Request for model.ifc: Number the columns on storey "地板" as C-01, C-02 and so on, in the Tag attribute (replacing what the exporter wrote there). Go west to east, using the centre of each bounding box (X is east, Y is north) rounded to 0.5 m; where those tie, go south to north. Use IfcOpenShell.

First a look at what the model holds.

```python
import ifcopenshell
import ifcopenshell.util.element
import ifcopenshell.util.placement

model = ifcopenshell.open("model.ifc")
print(model.schema)
storey = next(s for s in model.by_type("IfcBuildingStorey") if s.Name == "地板")
columns = [e for e in ifcopenshell.util.element.get_decomposition(storey) if e.is_a("IfcColumn")]
for e in sorted(columns, key=lambda e: e.id()):
    origin = ifcopenshell.util.placement.get_local_placement(e.ObjectPlacement)[:3, 3]
    print(e.id(), e.Tag, e.Name, origin.round(2) + 0.0, sep=" | ")
```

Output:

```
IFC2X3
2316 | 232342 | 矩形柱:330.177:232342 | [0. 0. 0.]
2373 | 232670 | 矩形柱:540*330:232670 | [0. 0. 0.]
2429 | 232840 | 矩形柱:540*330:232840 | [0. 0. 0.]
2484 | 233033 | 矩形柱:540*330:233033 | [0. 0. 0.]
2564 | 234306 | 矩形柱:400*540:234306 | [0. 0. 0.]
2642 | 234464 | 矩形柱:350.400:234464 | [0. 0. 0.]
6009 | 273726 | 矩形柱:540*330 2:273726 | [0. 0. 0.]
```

```python
import ifcopenshell
import ifcopenshell.geom
import ifcopenshell.util.element
import ifcopenshell.util.shape

model = ifcopenshell.open("model.ifc")
settings = ifcopenshell.geom.settings()
settings.set("use-world-coords", True)


def centre(element):
    shape = ifcopenshell.geom.create_shape(settings, element)
    return ifcopenshell.util.shape.get_bbox_centroid(shape.geometry)


storey = next(s for s in model.by_type("IfcBuildingStorey") if s.Name == "地板")
columns = [e for e in ifcopenshell.util.element.get_decomposition(storey) if e.is_a("IfcColumn")]

# Insertion points can sit at a corner or the storey origin, so sort by the geometry (in metres).
centres = {e: centre(e) for e in columns}
columns.sort(key=lambda e: (round(centres[e][0] / 0.5), centres[e][1]))

for i, e in enumerate(columns, start=1):
    number = f"C-{i:02d}"
    e.Tag = number
    print(e.id(), number)

model.write("model_updated.ifc")
```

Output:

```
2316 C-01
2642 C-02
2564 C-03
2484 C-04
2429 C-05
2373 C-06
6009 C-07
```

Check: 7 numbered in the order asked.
